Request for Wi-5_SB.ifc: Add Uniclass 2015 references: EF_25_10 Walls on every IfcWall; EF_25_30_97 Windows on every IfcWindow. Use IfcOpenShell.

First a look at what the model holds.

```python
import ifcopenshell

model = ifcopenshell.open("Wi-5_SB.ifc")
print(model.schema)
print("classifications:", [c.Name for c in model.by_type("IfcClassification")])
for ifc_class in ("IfcDoor", "IfcRoof", "IfcStair", "IfcWall", "IfcWindow"):
    print(ifc_class, len(model.by_type(ifc_class)))
```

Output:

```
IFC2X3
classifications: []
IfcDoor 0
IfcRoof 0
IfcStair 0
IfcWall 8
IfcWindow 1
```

```python
import ifcopenshell
import ifcopenshell.api.classification

model = ifcopenshell.open("Wi-5_SB.ifc")

# IFC2X3 requires Source and Edition and has no link from the project to the system.
system = model.create_entity("IfcClassification", Source="NBS", Edition="2015", Name="Uniclass 2015")

codes = {
    "IfcWall": ("EF_25_10", "Walls"),
    "IfcWindow": ("EF_25_30_97", "Windows"),
}
for ifc_class, (code, name) in codes.items():
    products = model.by_type(ifc_class)
    ifcopenshell.api.classification.add_reference(
        model, products=products, classification=system, identification=code, name=name
    )
    print(code, len(products))

model.write("Wi-5_SB_rev.ifc")
```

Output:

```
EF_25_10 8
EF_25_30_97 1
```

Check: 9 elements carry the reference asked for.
